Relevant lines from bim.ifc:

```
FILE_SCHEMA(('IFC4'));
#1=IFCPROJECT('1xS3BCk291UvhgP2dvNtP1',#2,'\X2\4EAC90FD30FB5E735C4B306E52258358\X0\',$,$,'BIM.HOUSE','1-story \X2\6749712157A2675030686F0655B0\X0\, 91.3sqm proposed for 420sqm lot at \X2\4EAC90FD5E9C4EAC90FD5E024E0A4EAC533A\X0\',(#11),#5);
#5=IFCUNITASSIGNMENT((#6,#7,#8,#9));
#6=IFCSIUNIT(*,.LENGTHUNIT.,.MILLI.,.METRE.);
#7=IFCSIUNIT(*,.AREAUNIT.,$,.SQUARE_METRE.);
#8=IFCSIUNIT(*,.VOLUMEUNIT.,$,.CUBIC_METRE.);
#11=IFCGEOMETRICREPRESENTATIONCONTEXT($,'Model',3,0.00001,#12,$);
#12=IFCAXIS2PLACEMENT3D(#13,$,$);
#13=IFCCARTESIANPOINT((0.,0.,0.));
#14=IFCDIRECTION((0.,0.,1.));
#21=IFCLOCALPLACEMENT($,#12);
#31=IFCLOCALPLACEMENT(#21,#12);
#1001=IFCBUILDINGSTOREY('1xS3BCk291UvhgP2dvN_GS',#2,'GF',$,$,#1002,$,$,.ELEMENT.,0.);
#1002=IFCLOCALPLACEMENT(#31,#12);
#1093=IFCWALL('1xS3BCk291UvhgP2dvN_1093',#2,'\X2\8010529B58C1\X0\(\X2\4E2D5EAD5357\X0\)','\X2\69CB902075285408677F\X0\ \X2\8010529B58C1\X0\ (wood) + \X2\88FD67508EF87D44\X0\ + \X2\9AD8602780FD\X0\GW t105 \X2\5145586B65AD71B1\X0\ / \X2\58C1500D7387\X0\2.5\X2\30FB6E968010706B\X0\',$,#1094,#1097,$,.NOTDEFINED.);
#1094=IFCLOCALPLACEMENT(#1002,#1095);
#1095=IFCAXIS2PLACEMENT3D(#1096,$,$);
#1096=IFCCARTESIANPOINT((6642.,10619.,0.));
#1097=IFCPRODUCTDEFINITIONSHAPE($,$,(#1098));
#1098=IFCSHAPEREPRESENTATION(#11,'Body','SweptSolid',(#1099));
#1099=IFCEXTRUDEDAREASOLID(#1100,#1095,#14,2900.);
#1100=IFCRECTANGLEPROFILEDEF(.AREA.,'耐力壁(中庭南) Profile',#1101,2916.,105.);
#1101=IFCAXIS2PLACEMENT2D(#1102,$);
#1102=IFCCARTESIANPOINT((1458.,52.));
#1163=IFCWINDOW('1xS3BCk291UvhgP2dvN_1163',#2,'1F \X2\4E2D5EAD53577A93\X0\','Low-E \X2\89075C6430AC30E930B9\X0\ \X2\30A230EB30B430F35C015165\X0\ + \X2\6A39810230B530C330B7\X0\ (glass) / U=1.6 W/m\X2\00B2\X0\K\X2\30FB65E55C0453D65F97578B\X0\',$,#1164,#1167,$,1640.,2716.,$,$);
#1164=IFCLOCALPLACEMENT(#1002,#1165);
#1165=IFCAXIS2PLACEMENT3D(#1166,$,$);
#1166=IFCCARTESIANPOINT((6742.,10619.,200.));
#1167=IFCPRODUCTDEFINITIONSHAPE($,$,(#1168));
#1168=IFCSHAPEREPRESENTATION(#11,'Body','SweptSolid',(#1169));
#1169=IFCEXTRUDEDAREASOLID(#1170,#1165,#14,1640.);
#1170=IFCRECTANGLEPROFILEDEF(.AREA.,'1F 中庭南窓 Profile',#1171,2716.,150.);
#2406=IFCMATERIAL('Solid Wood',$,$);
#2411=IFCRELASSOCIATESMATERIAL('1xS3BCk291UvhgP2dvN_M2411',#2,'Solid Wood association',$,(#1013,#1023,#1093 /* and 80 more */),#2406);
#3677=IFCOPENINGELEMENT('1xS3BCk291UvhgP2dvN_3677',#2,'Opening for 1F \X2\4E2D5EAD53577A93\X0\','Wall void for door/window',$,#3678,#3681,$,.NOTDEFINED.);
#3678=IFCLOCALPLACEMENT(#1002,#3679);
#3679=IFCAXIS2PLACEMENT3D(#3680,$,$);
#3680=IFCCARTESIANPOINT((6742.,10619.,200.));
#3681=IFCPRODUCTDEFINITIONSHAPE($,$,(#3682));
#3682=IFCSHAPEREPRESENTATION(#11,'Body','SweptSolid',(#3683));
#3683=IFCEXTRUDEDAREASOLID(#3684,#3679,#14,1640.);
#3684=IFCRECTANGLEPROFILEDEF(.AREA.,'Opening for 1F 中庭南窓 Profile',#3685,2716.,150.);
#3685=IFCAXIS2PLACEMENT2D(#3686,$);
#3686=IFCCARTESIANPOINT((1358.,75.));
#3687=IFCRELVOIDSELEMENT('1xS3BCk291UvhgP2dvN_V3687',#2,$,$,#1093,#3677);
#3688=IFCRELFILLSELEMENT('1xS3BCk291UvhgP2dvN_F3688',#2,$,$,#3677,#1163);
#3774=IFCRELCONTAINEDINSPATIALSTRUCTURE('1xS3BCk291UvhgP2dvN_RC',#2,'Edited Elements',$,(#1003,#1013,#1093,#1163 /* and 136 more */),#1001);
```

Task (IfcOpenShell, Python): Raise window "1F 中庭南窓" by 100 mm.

```python
import numpy as np
import ifcopenshell
import ifcopenshell.api.geometry
import ifcopenshell.util.placement
import ifcopenshell.util.unit

model = ifcopenshell.open("bim.ifc")
unit_scale = ifcopenshell.util.unit.calculate_unit_scale(model)

window = model.by_guid("1xS3BCk291UvhgP2dvN_1163")
opening = window.FillsVoids[0].RelatingOpeningElement
dz = 100.0

shift = np.array([0.0, 0.0, dz])
# The window is not placed relative to its opening, so move both.
for product in (opening, window):
    matrix = ifcopenshell.util.placement.get_local_placement(product.ObjectPlacement)
    matrix[:3, 3] += shift
    ifcopenshell.api.geometry.edit_object_placement(model, product=product, matrix=matrix, is_si=False)

print(f"moved by {dz * unit_scale:+.3f} m")

model.write("bim_edited.ifc")
```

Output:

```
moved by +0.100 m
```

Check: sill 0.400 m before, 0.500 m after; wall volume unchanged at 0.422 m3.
